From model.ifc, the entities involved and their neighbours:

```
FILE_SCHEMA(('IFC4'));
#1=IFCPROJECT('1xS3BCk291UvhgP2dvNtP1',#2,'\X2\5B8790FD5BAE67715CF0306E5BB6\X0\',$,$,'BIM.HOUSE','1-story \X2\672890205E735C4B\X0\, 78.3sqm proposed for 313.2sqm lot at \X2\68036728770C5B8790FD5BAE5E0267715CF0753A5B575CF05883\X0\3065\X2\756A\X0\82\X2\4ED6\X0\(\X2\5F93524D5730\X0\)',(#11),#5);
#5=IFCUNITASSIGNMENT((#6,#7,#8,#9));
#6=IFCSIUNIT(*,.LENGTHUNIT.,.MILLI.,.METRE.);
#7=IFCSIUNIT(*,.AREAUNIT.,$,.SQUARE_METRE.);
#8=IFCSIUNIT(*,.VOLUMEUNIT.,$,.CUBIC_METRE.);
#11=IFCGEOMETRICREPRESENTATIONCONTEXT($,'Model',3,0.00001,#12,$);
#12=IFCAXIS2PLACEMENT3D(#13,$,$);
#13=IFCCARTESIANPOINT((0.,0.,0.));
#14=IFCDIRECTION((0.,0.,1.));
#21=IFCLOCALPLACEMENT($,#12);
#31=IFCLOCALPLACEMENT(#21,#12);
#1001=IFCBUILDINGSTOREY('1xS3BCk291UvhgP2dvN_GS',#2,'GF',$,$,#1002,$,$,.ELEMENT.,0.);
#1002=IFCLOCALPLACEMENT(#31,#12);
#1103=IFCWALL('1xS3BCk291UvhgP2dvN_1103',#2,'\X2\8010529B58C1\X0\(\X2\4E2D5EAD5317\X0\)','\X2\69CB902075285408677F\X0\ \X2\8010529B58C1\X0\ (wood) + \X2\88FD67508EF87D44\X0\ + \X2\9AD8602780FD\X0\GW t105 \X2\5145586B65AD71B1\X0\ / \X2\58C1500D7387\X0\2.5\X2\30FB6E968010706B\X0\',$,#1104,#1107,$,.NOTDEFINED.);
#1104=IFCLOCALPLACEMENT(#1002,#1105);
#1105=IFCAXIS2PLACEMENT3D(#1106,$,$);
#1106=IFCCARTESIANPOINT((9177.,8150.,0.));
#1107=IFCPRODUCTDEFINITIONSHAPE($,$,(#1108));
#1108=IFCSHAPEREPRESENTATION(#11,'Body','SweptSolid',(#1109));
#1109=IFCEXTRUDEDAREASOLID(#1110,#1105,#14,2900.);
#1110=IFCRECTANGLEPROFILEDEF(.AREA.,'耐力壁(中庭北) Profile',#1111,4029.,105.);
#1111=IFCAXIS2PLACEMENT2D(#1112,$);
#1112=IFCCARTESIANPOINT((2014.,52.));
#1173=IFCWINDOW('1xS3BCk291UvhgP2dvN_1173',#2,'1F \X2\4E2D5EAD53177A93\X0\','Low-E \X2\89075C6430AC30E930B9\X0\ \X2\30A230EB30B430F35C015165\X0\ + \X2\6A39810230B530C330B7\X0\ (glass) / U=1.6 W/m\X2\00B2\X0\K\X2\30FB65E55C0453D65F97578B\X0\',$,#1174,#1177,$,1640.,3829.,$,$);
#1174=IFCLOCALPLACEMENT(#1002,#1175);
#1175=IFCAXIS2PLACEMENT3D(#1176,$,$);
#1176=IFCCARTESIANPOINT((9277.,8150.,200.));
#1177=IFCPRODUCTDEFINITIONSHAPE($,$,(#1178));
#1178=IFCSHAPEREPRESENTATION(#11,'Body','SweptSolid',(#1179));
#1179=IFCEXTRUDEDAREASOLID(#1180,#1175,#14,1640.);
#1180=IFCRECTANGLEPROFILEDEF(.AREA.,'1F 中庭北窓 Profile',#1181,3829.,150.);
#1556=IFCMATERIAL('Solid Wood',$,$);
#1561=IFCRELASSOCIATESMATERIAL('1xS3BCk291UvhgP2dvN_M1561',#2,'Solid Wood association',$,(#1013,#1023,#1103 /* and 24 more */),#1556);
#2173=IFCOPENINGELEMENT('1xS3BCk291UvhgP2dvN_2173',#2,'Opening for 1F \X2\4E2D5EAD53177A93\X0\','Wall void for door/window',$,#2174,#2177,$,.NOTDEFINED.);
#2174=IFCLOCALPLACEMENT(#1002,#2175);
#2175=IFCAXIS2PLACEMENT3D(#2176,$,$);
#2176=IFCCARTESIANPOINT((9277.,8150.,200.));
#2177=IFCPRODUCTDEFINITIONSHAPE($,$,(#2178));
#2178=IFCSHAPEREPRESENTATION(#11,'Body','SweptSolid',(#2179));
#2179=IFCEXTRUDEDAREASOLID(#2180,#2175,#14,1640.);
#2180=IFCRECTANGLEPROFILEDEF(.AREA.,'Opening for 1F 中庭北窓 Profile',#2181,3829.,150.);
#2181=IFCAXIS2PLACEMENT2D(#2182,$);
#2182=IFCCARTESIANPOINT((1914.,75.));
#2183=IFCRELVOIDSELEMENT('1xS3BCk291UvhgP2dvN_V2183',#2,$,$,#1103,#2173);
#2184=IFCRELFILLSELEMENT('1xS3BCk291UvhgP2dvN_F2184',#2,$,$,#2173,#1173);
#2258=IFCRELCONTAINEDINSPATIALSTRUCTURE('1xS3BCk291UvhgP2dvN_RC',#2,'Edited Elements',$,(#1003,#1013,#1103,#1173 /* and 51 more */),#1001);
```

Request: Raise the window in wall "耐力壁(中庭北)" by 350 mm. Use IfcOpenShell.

```python
import numpy as np
import ifcopenshell
import ifcopenshell.api.geometry
import ifcopenshell.util.placement
import ifcopenshell.util.unit

model = ifcopenshell.open("model.ifc")
unit_scale = ifcopenshell.util.unit.calculate_unit_scale(model)

window = model.by_guid("1xS3BCk291UvhgP2dvN_1173")
opening = window.FillsVoids[0].RelatingOpeningElement
dz = 350.0

shift = np.array([0.0, 0.0, dz])
# The window is not placed relative to its opening, so move both.
for product in (opening, window):
    matrix = ifcopenshell.util.placement.get_local_placement(product.ObjectPlacement)
    matrix[:3, 3] += shift
    ifcopenshell.api.geometry.edit_object_placement(model, product=product, matrix=matrix, is_si=False)

print(f"moved by {dz * unit_scale:+.3f} m")

model.write("model_updated.ifc")
```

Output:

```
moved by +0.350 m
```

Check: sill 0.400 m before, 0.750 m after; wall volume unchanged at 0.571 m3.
